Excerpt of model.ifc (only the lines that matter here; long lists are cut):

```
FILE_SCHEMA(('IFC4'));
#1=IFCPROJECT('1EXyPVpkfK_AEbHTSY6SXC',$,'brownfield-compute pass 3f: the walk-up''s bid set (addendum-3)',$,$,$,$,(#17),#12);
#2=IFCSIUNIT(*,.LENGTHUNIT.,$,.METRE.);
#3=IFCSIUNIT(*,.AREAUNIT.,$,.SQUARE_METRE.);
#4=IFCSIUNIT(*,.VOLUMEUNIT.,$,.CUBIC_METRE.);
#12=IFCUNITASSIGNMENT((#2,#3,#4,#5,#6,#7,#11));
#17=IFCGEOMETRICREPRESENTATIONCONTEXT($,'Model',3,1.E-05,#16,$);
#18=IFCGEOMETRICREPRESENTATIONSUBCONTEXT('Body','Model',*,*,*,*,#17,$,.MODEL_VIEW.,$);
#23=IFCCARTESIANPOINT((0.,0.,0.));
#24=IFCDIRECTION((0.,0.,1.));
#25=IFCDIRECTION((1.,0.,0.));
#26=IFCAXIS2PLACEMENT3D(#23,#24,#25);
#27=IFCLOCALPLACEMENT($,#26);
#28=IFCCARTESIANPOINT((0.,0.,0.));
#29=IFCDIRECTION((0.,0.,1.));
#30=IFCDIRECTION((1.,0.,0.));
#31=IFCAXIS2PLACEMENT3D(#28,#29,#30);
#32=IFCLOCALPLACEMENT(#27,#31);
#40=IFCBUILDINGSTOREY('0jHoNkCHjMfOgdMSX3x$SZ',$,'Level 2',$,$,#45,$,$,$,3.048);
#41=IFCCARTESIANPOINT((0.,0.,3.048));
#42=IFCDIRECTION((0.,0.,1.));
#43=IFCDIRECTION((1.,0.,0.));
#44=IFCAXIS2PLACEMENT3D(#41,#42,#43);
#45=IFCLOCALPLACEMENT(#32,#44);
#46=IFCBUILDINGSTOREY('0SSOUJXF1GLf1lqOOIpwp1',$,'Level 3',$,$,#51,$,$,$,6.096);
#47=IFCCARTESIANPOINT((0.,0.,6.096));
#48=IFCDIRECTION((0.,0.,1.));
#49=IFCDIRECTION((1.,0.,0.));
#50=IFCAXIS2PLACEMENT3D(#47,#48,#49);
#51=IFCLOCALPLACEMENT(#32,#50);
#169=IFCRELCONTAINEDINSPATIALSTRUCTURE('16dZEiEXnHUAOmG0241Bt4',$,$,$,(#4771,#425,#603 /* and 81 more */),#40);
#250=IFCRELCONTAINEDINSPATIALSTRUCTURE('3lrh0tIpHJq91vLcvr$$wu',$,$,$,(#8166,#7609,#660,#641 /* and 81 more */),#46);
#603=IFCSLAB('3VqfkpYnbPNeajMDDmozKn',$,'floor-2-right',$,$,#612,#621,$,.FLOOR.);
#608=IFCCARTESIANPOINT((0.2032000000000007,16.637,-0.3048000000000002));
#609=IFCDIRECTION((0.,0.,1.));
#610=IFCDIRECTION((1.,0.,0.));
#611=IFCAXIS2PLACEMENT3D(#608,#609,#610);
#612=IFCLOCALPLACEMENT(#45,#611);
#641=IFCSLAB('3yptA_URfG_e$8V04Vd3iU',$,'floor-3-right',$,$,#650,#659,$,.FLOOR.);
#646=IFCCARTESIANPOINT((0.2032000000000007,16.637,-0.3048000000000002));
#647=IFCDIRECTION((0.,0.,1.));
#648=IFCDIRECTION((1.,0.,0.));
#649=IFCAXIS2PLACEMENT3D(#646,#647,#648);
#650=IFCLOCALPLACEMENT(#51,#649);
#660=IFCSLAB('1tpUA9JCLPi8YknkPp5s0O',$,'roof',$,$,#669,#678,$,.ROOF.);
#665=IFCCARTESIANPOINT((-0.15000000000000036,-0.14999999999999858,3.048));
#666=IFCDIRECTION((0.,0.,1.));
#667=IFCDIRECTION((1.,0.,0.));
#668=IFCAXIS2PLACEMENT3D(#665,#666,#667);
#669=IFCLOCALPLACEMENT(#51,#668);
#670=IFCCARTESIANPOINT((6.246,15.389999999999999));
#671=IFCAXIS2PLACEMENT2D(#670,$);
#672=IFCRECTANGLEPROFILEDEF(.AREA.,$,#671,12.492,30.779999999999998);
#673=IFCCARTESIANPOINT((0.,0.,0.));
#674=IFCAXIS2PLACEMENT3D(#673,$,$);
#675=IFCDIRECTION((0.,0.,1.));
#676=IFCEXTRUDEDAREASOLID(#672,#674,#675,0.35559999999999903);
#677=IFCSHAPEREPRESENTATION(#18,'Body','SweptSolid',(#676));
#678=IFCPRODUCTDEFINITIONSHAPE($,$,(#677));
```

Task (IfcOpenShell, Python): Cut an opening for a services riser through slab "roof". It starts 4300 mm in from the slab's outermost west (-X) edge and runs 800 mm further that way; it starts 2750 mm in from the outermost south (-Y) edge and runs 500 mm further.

```python
import numpy as np
import ifcopenshell
import ifcopenshell.api.feature
import ifcopenshell.api.geometry
import ifcopenshell.api.root
import ifcopenshell.geom
import ifcopenshell.util.placement
import ifcopenshell.util.representation
import ifcopenshell.util.shape
import ifcopenshell.util.unit

model = ifcopenshell.open("model.ifc")
unit_scale = ifcopenshell.util.unit.calculate_unit_scale(model)
settings = ifcopenshell.geom.settings()


def volume(element):
    """Net volume in cubic metres, openings subtracted."""
    shape = ifcopenshell.geom.create_shape(settings, element)
    return ifcopenshell.util.shape.get_volume(shape.geometry)


slab = model.by_guid("1tpUA9JCLPi8YknkPp5s0O")
before = volume(slab)

# Extent in the slab's own axes, in metres. The edges named are its -X and -Y sides.
slab_shape = ifcopenshell.geom.create_shape(settings, slab)
vertices = ifcopenshell.util.shape.get_vertices(slab_shape.geometry)
x_min, y_min, bottom = vertices.min(axis=0)
top = vertices[:, 2].max()

opening = ifcopenshell.api.root.create_entity(model, ifc_class="IfcOpeningElement", name="Services riser opening", predefined_type="OPENING")
context = ifcopenshell.util.representation.get_context(model, "Model", "Body", "MODEL_VIEW")
width, depth = 0.8, 0.5
outline = [(0.0, 0.0), (width, 0.0), (width, depth), (0.0, depth), (0.0, 0.0)]
# Overshoot both faces by 50 mm so the cut is clean.
shape = ifcopenshell.api.geometry.add_slab_representation(
    model, context=context, depth=top - bottom + 0.1, polyline=outline
)
ifcopenshell.api.geometry.assign_representation(model, product=opening, representation=shape)

matrix = ifcopenshell.util.placement.get_local_placement(slab.ObjectPlacement)
matrix[:, 3] = matrix @ np.append(np.array([x_min + 4.3, y_min + 2.75, bottom - 0.05]) / unit_scale, 1.0)
ifcopenshell.api.geometry.edit_object_placement(model, product=opening, matrix=matrix, is_si=False)
ifcopenshell.api.feature.add_feature(model, feature=opening, element=slab)

after = volume(slab)

print(f"slab volume {before:.3f} -> {after:.3f} m3")

model.write("model_rev.ifc")
```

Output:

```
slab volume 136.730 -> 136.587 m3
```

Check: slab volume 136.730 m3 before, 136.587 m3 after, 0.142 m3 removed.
